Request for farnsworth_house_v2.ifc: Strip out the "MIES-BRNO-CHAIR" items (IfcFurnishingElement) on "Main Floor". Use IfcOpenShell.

First a look at what the model holds.

```python
import ifcopenshell
import ifcopenshell.util.element

model = ifcopenshell.open("farnsworth_house_v2.ifc")
print(model.schema)
storey = next(s for s in model.by_type("IfcBuildingStorey") if s.Name == "Main Floor")
furniture = [e for e in ifcopenshell.util.element.get_decomposition(storey) if e.is_a("IfcFurnishingElement")]
seen = {}
for e in furniture:
    element_type = ifcopenshell.util.element.get_type(e)
    name = element_type.Name if element_type not in (None, e) else None
    seen[name] = seen.get(name, 0) + 1
for name, count in sorted(seen.items(), key=str):
    print(count, "x", name)
```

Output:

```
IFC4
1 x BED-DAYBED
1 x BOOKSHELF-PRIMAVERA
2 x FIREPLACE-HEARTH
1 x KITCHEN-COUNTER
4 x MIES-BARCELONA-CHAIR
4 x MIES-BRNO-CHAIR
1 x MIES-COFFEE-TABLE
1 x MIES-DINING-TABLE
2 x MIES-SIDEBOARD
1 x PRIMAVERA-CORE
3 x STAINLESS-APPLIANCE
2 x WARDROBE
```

```python
import ifcopenshell
import ifcopenshell.api.root
import ifcopenshell.util.element

model = ifcopenshell.open("farnsworth_house_v2.ifc")

storey = next(s for s in model.by_type("IfcBuildingStorey") if s.Name == "Main Floor")
furniture = [e for e in ifcopenshell.util.element.get_decomposition(storey) if e.is_a("IfcFurnishingElement")]
targets = [e for e in furniture if (t := ifcopenshell.util.element.get_type(e)) not in (None, e) and t.Name == "MIES-BRNO-CHAIR"]

for e in targets:
    ifcopenshell.api.root.remove_product(model, product=e)
print(len(targets), "removed")

model.write("farnsworth_house_v2_updated.ifc")
```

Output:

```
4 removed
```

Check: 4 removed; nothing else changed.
